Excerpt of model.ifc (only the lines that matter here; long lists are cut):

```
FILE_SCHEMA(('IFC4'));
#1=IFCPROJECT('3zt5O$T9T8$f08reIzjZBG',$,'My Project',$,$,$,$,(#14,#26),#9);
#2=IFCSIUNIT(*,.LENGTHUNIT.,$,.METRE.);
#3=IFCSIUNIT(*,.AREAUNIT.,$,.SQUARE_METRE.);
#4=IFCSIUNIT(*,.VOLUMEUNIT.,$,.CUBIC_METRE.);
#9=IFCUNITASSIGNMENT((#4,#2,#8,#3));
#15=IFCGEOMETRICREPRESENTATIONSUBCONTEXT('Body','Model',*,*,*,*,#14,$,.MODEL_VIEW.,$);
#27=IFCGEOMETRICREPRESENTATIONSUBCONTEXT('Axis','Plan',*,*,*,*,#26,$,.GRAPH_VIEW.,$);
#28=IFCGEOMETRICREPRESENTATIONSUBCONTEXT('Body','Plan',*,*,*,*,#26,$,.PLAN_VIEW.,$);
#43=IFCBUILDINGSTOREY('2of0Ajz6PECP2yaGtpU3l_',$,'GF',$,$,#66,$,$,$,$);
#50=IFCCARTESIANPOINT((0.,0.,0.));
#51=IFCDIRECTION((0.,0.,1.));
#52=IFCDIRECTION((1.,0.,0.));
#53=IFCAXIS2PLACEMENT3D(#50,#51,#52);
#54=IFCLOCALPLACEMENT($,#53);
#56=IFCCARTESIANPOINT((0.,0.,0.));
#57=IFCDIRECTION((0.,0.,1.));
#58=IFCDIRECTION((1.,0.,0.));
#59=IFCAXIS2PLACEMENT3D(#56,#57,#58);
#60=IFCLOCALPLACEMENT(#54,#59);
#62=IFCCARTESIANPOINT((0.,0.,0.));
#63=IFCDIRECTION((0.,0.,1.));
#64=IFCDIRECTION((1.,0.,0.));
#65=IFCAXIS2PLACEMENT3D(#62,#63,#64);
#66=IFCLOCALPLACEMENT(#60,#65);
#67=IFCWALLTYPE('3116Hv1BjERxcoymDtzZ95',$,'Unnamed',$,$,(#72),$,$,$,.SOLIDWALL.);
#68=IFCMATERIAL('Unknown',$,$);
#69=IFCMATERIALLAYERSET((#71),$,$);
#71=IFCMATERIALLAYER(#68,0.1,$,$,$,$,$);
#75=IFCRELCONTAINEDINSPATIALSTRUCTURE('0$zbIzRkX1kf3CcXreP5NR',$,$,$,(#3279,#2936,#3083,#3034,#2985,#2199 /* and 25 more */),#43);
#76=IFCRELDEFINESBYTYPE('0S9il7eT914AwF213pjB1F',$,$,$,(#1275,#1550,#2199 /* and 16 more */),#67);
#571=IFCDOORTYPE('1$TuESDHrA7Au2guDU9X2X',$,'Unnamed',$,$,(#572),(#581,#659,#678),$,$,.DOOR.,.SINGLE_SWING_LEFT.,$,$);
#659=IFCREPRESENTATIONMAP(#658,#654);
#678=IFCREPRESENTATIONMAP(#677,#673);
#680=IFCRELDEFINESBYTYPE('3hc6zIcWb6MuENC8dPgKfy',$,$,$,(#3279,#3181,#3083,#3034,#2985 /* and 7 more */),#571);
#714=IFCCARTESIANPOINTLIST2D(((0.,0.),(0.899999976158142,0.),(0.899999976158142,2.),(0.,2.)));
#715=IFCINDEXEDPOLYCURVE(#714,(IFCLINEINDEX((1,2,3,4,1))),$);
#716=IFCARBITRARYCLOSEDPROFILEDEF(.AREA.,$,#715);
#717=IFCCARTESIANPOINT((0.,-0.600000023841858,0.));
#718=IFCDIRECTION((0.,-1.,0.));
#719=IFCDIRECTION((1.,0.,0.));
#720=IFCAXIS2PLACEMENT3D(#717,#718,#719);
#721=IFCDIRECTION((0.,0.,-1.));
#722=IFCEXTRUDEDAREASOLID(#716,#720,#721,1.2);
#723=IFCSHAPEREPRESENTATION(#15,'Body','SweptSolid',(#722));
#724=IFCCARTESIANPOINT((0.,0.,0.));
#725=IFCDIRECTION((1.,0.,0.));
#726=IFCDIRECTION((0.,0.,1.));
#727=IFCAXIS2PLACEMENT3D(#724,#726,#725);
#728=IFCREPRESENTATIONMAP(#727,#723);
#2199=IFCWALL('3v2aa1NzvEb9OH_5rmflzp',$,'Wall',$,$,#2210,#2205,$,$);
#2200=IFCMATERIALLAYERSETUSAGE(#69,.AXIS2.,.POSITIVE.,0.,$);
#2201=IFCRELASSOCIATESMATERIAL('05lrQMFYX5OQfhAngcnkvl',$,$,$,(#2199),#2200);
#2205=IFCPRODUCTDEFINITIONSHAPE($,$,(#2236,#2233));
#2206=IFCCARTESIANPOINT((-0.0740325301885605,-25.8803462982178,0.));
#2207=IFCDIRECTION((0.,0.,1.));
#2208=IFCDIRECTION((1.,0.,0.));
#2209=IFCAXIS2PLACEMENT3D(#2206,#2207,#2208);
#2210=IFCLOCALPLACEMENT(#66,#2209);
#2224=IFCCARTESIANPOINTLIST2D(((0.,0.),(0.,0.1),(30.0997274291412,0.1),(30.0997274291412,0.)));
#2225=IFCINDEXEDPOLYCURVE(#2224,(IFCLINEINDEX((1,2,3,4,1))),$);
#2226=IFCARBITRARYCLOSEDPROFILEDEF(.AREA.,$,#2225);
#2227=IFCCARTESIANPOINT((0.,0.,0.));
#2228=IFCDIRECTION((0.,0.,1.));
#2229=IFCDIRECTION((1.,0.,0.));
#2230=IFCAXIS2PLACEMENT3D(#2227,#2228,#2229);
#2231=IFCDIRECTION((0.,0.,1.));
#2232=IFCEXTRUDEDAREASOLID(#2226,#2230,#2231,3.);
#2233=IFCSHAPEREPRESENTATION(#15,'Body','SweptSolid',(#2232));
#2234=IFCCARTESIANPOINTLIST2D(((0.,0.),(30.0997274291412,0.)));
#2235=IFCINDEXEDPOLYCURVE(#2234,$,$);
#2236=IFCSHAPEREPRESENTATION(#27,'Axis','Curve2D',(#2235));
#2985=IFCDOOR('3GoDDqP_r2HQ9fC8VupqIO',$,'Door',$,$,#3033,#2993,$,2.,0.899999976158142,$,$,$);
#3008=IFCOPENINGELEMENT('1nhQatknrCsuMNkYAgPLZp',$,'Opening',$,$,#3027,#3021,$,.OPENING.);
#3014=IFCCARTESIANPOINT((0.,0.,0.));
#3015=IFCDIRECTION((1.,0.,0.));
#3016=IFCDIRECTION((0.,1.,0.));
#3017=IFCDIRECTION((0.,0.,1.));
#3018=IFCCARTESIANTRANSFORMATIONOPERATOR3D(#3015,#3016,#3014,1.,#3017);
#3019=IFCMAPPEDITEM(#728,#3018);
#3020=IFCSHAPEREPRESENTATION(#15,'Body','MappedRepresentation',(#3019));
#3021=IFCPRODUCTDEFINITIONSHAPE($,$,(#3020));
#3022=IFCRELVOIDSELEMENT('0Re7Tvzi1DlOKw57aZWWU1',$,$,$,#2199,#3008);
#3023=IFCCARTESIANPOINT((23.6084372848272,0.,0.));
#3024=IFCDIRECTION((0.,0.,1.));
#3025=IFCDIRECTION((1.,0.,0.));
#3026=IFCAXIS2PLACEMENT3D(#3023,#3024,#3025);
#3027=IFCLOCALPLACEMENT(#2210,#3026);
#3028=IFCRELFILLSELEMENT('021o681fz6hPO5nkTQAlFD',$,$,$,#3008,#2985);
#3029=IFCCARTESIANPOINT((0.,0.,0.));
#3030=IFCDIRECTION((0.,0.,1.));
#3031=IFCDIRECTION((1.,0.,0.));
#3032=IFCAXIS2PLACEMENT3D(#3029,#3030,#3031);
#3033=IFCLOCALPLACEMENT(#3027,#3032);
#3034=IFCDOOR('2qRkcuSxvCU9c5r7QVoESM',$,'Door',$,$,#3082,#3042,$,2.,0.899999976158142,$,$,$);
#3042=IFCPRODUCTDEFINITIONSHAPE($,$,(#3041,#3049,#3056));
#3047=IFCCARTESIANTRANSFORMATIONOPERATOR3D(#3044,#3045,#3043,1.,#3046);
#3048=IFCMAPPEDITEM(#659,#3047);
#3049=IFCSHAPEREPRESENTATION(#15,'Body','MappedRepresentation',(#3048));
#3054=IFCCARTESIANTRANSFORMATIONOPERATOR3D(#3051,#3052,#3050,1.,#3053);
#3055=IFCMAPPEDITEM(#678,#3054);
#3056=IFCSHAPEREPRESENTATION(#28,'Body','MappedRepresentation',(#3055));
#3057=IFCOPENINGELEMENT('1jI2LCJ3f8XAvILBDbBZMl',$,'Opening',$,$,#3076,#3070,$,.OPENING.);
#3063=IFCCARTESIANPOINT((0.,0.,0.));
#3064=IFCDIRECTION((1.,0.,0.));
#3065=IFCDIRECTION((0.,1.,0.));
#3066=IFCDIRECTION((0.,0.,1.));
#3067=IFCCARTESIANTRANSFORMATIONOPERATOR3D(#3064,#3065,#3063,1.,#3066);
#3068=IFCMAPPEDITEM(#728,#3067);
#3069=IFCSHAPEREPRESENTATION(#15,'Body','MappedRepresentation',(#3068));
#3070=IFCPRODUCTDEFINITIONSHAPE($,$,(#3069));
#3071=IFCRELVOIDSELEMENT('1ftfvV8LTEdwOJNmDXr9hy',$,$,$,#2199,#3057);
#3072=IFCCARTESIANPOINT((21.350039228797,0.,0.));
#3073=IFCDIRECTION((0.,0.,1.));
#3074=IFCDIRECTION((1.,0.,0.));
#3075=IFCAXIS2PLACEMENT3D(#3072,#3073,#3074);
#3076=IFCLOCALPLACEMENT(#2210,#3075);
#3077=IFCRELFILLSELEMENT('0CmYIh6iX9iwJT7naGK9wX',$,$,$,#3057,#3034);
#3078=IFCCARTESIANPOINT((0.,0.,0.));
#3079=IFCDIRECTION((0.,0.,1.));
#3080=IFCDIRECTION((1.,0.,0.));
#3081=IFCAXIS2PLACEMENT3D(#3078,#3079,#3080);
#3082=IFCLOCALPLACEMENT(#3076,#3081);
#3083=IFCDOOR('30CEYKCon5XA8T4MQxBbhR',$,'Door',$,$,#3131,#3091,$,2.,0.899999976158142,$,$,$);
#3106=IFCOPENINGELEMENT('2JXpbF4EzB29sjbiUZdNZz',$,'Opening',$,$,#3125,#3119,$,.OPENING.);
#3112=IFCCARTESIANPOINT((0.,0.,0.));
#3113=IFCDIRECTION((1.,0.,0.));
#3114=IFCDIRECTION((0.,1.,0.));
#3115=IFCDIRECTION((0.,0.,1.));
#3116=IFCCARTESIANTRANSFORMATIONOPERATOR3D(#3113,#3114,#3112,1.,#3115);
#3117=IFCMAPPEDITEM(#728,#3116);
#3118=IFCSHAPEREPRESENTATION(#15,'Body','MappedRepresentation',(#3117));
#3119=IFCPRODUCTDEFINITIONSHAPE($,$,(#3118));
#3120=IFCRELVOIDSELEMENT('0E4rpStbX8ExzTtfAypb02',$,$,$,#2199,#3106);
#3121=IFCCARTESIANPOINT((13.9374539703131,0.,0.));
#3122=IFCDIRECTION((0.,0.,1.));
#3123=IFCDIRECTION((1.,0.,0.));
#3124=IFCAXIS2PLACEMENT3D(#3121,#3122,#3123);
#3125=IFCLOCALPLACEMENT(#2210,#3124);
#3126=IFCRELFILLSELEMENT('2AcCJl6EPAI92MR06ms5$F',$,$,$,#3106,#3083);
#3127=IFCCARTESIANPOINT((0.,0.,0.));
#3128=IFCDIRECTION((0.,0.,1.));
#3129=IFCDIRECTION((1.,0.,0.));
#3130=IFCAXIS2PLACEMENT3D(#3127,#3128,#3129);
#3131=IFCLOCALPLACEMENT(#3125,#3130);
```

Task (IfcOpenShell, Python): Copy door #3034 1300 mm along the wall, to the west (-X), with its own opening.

```python
import ifcopenshell
import ifcopenshell.api.feature
import ifcopenshell.api.geometry
import ifcopenshell.api.root
import ifcopenshell.geom
import ifcopenshell.util.element
import ifcopenshell.util.placement
import ifcopenshell.util.shape

model = ifcopenshell.open("model.ifc")
settings = ifcopenshell.geom.settings()


def volume(element):
    """Net volume in cubic metres, openings subtracted."""
    shape = ifcopenshell.geom.create_shape(settings, element)
    return ifcopenshell.util.shape.get_volume(shape.geometry)


door = model.by_guid("2qRkcuSxvCU9c5r7QVoESM")
opening = door.FillsVoids[0].RelatingOpeningElement
wall = opening.VoidsElements[0].RelatingBuildingElement
before = volume(wall)
shift = ifcopenshell.util.placement.get_local_placement(wall.ObjectPlacement)[:3, 0] * -1.3

# copy_class copies the void relationship, type, container and properties, but no geometry.
new_opening = ifcopenshell.api.root.copy_class(model, product=opening)
new_opening.Representation = ifcopenshell.util.element.copy_deep(
    model, opening.Representation, exclude=["IfcGeometricRepresentationContext", "IfcRepresentationMap"]
)
new_door = ifcopenshell.api.root.copy_class(model, product=door)
new_door.Representation = ifcopenshell.util.element.copy_deep(
    model, door.Representation, exclude=["IfcGeometricRepresentationContext", "IfcRepresentationMap"]
)
ifcopenshell.api.feature.add_filling(model, opening=new_opening, element=new_door)

for old, new in ((opening, new_opening), (door, new_door)):
    matrix = ifcopenshell.util.placement.get_local_placement(old.ObjectPlacement)
    matrix[:3, 3] += shift
    ifcopenshell.api.geometry.edit_object_placement(model, product=new, matrix=matrix, is_si=False)

after = volume(wall)

print(f"wall volume {before:.3f} -> {after:.3f} m3")

model.write("model_v2.ifc")
```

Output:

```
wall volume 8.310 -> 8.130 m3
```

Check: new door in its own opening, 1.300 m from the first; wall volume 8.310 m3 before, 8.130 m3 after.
